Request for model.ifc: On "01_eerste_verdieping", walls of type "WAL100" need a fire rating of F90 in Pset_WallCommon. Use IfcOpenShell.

First a look at what the model holds.

```python
import ifcopenshell
import ifcopenshell.util.element

model = ifcopenshell.open("model.ifc")
print(model.schema)
storey = next(s for s in model.by_type("IfcBuildingStorey") if s.Name == "01_eerste_verdieping")
walls = [e for e in ifcopenshell.util.element.get_decomposition(storey) if e.is_a("IfcWall")]
seen = {}
for e in walls:
    element_type = ifcopenshell.util.element.get_type(e)
    key = (element_type.Name if element_type != e and element_type else None, ifcopenshell.util.element.get_pset(e, "Pset_WallCommon", "FireRating"))
    seen[key] = seen.get(key, 0) + 1
for (name, value), count in sorted(seen.items(), key=str):
    print(count, "x", name, "|", value)
```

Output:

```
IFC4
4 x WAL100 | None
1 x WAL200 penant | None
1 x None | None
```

```python
import ifcopenshell
import ifcopenshell.api.pset
import ifcopenshell.util.element

model = ifcopenshell.open("model.ifc")

storey = next(s for s in model.by_type("IfcBuildingStorey") if s.Name == "01_eerste_verdieping")
walls = [e for e in ifcopenshell.util.element.get_decomposition(storey) if e.is_a("IfcWall")]

count = 0
for e in walls:
    element_type = ifcopenshell.util.element.get_type(e)
    if element_type in (None, e) or element_type.Name != "WAL100":
        continue
    # add_pset returns the element's existing set when there is one.
    pset = ifcopenshell.api.pset.add_pset(model, product=e, name="Pset_WallCommon")
    ifcopenshell.api.pset.edit_pset(model, pset=pset, properties={"FireRating": "F90"})
    count += 1

print(count, "walls updated")

model.write("model_v2.ifc")
```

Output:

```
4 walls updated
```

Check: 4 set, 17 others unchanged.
